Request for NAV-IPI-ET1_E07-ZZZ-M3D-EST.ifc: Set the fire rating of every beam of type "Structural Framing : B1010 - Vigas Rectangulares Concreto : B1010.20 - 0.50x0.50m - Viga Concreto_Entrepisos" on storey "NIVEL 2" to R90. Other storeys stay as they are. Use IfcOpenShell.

First a look at what the model holds.

```python
import ifcopenshell
import ifcopenshell.util.element

model = ifcopenshell.open("NAV-IPI-ET1_E07-ZZZ-M3D-EST.ifc")
print(model.schema)
storey = next(s for s in model.by_type("IfcBuildingStorey") if s.Name == "NIVEL 2")
beams = [e for e in ifcopenshell.util.element.get_decomposition(storey) if e.is_a("IfcBeam")]
seen = {}
for e in beams:
    element_type = ifcopenshell.util.element.get_type(e)
    key = (element_type.Name if element_type != e and element_type else None, ifcopenshell.util.element.get_pset(e, "Pset_BeamCommon", "FireRating"))
    seen[key] = seen.get(key, 0) + 1
for (name, value), count in sorted(seen.items(), key=str):
    print(count, "x", name, "|", value)
```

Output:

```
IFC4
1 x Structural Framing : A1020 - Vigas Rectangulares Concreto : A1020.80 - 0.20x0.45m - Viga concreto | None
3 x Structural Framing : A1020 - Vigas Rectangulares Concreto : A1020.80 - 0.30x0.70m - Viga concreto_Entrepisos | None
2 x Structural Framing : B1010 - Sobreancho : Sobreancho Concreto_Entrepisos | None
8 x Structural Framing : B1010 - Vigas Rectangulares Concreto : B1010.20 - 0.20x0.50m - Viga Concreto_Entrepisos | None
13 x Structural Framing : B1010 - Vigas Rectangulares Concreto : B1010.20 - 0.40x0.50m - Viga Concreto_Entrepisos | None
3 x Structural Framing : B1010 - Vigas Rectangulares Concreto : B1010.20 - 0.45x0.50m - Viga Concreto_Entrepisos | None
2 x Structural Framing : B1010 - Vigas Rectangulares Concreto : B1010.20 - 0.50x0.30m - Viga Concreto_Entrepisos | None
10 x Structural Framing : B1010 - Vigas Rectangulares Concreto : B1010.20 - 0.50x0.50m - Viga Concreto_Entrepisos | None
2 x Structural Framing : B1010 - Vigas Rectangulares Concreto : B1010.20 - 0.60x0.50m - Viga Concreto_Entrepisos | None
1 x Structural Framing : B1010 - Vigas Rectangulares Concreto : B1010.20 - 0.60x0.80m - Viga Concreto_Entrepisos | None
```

```python
import ifcopenshell
import ifcopenshell.api.pset
import ifcopenshell.util.element

model = ifcopenshell.open("NAV-IPI-ET1_E07-ZZZ-M3D-EST.ifc")

storey = next(s for s in model.by_type("IfcBuildingStorey") if s.Name == "NIVEL 2")
beams = [e for e in ifcopenshell.util.element.get_decomposition(storey) if e.is_a("IfcBeam")]

count = 0
for e in beams:
    element_type = ifcopenshell.util.element.get_type(e)
    if element_type in (None, e) or element_type.Name != "Structural Framing : B1010 - Vigas Rectangulares Concreto : B1010.20 - 0.50x0.50m - Viga Concreto_Entrepisos":
        continue
    # add_pset returns the element's existing set when there is one.
    pset = ifcopenshell.api.pset.add_pset(model, product=e, name="Pset_BeamCommon")
    ifcopenshell.api.pset.edit_pset(model, pset=pset, properties={"FireRating": "R90"})
    count += 1

print(count, "beams updated")

model.write("NAV-IPI-ET1_E07-ZZZ-M3D-EST_updated.ifc")
```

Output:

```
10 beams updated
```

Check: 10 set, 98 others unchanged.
